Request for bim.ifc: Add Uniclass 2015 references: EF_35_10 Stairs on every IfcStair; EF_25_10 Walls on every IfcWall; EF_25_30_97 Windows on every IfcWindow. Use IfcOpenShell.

First a look at what the model holds.

```python
import ifcopenshell

model = ifcopenshell.open("bim.ifc")
print(model.schema)
print("classifications:", [c.Name for c in model.by_type("IfcClassification")])
for ifc_class in ("IfcDoor", "IfcRoof", "IfcStair", "IfcWall", "IfcWindow"):
    print(ifc_class, len(model.by_type(ifc_class)))
```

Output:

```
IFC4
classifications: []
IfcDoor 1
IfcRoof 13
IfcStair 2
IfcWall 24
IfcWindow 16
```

```python
import ifcopenshell
import ifcopenshell.api.classification

model = ifcopenshell.open("bim.ifc")

system = ifcopenshell.api.classification.add_classification(model, classification="Uniclass 2015")

codes = {
    "IfcStair": ("EF_35_10", "Stairs"),
    "IfcWall": ("EF_25_10", "Walls"),
    "IfcWindow": ("EF_25_30_97", "Windows"),
}
for ifc_class, (code, name) in codes.items():
    products = model.by_type(ifc_class)
    ifcopenshell.api.classification.add_reference(
        model, products=products, classification=system, identification=code, name=name
    )
    print(code, len(products))

model.write("bim_rev.ifc")
```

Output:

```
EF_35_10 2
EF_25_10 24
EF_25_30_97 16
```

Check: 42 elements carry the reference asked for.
